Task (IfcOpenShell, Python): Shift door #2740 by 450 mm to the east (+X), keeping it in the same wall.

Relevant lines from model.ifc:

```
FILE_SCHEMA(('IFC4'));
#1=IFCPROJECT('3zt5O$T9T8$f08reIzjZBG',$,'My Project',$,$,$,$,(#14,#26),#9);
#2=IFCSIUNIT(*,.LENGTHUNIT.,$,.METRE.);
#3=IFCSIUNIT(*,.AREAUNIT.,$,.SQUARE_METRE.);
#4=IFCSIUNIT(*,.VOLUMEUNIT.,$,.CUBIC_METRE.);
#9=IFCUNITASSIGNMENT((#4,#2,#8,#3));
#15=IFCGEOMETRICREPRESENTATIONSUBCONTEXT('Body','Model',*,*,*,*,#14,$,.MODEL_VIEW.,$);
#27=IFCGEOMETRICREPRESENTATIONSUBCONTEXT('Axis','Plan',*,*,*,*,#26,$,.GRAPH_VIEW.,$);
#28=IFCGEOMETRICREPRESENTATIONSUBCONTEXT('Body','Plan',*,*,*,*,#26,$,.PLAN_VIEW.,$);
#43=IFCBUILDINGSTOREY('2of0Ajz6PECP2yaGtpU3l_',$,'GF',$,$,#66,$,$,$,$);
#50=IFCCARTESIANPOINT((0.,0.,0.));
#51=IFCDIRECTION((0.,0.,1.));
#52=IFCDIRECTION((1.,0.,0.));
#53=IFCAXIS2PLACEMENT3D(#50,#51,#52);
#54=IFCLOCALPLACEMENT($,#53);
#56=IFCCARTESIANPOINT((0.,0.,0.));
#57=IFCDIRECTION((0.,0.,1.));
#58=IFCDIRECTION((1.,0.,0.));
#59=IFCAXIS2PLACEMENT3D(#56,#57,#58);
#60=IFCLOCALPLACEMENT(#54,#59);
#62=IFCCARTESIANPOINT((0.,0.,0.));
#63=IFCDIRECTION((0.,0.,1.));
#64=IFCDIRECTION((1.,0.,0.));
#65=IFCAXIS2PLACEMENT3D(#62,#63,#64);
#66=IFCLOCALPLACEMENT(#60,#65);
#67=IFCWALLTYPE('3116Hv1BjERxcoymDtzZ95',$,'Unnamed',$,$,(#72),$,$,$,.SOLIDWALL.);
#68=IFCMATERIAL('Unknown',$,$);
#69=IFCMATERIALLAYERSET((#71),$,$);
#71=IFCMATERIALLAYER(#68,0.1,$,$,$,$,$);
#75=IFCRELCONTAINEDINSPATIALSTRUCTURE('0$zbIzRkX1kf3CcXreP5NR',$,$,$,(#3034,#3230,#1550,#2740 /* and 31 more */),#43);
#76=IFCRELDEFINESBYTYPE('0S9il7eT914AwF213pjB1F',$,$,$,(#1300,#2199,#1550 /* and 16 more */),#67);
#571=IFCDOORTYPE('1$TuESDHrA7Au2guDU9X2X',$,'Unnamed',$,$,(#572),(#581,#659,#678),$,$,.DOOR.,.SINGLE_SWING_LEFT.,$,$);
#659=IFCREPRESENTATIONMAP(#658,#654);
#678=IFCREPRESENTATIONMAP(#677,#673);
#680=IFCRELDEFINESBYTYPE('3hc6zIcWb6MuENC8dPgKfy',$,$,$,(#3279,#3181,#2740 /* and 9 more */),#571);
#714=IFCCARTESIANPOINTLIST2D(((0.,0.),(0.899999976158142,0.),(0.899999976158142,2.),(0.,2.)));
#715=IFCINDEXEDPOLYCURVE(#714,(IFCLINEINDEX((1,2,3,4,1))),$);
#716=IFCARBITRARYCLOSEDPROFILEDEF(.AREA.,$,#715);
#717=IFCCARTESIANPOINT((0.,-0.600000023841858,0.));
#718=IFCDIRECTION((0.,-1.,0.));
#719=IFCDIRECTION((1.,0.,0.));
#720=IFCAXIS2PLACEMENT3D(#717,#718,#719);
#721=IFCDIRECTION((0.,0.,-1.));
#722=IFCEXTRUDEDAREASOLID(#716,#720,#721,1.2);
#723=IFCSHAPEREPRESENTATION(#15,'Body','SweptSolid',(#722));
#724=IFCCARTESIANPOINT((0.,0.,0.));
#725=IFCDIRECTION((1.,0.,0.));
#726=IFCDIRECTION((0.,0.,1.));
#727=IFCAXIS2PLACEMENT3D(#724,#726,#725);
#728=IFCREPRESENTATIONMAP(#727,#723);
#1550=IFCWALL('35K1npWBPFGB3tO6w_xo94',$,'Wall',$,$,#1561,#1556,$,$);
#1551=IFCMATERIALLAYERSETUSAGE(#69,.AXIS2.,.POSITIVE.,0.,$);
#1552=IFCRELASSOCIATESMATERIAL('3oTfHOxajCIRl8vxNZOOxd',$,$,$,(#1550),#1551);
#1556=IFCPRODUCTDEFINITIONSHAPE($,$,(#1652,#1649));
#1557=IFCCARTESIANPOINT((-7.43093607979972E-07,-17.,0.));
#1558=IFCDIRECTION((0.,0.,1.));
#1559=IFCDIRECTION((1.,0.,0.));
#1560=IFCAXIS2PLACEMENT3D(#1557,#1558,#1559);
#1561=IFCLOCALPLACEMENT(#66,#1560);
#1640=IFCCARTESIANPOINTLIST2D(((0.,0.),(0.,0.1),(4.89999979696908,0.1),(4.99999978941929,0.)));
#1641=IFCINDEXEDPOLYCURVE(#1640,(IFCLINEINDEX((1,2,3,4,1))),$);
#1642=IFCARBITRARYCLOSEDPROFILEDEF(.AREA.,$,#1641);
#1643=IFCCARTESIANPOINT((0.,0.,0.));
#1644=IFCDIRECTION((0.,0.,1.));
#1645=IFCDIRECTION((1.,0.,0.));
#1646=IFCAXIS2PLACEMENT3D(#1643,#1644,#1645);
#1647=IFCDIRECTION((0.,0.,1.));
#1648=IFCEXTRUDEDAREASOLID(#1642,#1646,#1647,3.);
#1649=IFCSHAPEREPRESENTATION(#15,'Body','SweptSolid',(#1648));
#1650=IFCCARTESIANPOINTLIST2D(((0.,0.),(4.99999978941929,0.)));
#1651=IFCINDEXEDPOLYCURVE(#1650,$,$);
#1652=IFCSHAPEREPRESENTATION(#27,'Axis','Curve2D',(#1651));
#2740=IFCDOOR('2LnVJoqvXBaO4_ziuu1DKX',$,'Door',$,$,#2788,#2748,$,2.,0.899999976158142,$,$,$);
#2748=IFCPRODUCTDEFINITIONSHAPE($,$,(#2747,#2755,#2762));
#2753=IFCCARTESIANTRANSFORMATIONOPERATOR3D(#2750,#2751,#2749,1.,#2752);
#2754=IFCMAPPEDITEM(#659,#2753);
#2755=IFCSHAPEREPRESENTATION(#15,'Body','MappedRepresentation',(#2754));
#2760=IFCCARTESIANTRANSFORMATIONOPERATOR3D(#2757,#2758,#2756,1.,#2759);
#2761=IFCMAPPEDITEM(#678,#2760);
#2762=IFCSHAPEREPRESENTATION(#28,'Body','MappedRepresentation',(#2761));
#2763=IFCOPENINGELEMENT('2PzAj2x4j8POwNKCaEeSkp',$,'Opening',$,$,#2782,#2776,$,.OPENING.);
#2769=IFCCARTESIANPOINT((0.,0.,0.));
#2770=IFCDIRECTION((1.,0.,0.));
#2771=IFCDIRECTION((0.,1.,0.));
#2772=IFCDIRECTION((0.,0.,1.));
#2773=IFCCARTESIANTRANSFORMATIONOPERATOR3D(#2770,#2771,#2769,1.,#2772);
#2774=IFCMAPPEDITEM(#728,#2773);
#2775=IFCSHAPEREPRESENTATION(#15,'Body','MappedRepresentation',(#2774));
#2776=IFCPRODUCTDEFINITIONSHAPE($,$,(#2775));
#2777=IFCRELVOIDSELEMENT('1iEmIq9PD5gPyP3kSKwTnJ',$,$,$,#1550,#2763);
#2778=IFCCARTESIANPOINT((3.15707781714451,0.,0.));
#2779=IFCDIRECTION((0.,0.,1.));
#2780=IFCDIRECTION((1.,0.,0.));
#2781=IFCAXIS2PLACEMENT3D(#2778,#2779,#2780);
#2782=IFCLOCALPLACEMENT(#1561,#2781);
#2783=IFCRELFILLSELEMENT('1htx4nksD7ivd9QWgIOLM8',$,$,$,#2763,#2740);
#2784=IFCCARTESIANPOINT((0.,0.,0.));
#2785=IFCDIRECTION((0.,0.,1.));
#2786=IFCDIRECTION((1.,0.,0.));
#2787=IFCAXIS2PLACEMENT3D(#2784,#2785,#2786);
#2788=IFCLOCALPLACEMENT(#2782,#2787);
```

```python
import ifcopenshell
import ifcopenshell.api.geometry
import ifcopenshell.util.placement
import ifcopenshell.util.unit

model = ifcopenshell.open("model.ifc")
unit_scale = ifcopenshell.util.unit.calculate_unit_scale(model)

door = model.by_guid("2LnVJoqvXBaO4_ziuu1DKX")
opening = door.FillsVoids[0].RelatingOpeningElement
wall = opening.VoidsElements[0].RelatingBuildingElement

wall_matrix = ifcopenshell.util.placement.get_local_placement(wall.ObjectPlacement)
shift = wall_matrix[:3, 0] * 0.45 / unit_scale
before = ifcopenshell.util.placement.get_local_placement(door.ObjectPlacement)[:3, 3].copy()

# The door is placed relative to its opening, so it follows when the opening moves.
matrix = ifcopenshell.util.placement.get_local_placement(opening.ObjectPlacement)
matrix[:3, 3] += shift
ifcopenshell.api.geometry.edit_object_placement(
    model, product=opening, matrix=matrix, is_si=False, should_transform_children=True
)

after = ifcopenshell.util.placement.get_local_placement(door.ObjectPlacement)[:3, 3]
print("door moved by", (after - before).round(3) + 0.0)

model.write("model_v2.ifc")
```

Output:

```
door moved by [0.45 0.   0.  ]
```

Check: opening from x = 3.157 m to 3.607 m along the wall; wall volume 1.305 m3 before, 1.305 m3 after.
